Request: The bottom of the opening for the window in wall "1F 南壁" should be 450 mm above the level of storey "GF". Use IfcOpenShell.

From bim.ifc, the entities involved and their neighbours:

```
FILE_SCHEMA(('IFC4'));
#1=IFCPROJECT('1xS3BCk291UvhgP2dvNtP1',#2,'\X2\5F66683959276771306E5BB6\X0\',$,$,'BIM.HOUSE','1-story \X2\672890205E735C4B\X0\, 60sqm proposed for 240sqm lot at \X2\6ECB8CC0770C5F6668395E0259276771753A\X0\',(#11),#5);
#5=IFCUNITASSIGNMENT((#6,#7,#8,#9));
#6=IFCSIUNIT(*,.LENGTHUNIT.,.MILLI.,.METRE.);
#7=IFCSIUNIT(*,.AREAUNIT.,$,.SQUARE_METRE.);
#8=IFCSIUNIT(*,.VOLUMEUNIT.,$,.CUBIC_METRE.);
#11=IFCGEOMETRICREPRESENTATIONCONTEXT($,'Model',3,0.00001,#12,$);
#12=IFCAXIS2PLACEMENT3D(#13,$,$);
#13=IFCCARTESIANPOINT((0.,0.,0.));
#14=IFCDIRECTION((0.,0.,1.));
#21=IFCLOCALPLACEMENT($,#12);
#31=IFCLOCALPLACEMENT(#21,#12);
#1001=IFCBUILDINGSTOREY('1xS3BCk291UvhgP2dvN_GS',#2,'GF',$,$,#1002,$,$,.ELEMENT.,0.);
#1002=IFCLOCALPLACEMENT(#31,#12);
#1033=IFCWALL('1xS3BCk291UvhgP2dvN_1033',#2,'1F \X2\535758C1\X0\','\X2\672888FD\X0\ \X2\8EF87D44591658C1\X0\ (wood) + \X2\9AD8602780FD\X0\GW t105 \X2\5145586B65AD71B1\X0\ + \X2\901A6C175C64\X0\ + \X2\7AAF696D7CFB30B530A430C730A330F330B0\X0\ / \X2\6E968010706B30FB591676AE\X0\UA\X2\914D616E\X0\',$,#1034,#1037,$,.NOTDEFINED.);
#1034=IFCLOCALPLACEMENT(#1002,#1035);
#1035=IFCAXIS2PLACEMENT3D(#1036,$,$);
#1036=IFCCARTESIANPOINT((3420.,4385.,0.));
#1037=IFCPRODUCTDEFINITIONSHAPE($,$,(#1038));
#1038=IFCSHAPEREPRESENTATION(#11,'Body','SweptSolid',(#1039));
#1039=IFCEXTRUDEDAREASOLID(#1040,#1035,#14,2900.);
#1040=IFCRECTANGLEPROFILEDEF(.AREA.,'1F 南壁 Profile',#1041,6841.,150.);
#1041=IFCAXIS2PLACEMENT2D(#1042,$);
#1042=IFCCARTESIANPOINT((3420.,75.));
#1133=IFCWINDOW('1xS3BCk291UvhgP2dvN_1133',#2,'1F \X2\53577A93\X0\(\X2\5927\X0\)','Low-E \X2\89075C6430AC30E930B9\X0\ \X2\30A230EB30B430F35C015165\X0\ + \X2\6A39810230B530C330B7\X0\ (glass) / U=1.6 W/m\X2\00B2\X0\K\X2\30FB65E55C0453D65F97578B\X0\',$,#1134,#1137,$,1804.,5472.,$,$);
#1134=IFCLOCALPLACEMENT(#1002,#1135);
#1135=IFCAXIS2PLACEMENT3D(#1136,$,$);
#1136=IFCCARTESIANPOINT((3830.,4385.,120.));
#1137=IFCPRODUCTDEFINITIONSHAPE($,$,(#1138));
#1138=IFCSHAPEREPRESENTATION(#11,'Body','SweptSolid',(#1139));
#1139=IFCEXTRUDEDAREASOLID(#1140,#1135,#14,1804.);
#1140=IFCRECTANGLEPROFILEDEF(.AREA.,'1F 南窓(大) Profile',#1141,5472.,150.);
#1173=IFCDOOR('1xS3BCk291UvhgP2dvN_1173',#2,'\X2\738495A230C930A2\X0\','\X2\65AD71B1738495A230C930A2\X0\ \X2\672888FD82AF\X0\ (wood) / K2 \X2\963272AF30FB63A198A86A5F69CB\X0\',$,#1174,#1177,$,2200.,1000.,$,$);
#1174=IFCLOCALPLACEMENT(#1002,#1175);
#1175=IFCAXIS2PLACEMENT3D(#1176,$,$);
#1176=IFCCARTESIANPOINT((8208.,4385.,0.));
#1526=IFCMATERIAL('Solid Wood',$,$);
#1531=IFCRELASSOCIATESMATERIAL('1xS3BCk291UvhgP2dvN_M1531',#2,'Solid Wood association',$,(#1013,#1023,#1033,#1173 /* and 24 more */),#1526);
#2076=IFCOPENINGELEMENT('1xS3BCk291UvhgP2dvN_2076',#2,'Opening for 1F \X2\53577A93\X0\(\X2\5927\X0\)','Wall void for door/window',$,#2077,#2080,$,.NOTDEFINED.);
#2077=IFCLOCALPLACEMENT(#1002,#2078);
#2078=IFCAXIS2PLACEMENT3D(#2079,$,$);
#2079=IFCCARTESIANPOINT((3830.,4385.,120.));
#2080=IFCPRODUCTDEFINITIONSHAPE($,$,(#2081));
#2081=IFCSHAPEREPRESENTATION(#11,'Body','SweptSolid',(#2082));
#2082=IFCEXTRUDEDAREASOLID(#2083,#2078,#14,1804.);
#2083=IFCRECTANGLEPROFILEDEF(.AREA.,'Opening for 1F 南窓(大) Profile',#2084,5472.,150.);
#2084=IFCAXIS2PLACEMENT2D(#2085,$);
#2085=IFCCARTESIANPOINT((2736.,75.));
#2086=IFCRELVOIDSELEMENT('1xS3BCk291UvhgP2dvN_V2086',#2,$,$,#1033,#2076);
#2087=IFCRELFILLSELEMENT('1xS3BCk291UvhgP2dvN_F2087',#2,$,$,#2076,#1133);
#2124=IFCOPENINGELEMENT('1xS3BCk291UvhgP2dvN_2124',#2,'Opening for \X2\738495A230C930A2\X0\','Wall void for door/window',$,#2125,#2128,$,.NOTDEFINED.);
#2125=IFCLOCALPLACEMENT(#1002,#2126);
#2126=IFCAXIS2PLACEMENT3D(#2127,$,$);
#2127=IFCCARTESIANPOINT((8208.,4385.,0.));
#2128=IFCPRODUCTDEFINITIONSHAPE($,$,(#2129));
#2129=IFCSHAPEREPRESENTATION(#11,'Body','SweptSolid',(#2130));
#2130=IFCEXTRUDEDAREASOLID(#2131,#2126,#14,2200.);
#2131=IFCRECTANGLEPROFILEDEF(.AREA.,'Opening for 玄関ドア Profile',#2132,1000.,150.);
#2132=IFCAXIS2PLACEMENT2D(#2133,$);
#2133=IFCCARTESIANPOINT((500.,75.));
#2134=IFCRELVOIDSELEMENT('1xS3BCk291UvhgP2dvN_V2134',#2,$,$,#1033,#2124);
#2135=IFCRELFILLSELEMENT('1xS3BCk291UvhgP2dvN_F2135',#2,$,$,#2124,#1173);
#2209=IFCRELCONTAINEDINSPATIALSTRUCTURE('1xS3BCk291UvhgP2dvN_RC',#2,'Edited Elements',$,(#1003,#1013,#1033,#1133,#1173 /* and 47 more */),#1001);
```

```python
import numpy as np
import ifcopenshell
import ifcopenshell.api.geometry
import ifcopenshell.geom
import ifcopenshell.util.element
import ifcopenshell.util.placement
import ifcopenshell.util.shape
import ifcopenshell.util.unit

model = ifcopenshell.open("bim.ifc")
unit_scale = ifcopenshell.util.unit.calculate_unit_scale(model)

window = model.by_id(1133)
opening = window.FillsVoids[0].RelatingOpeningElement
storey = ifcopenshell.util.element.get_container(window, ifc_class="IfcBuildingStorey")
level = ifcopenshell.util.placement.get_local_placement(storey.ObjectPlacement)[2, 3]

# The opening's origin need not be at the sill, so measure its lowest point.
shape = ifcopenshell.geom.create_shape(ifcopenshell.geom.settings(), opening)
bottom = ifcopenshell.util.shape.get_shape_bottom_elevation(shape, shape.geometry) / unit_scale
dz = level + 0.45 / unit_scale - bottom

shift = np.array([0.0, 0.0, dz])
# The window is not placed relative to its opening, so move both.
for product in (opening, window):
    matrix = ifcopenshell.util.placement.get_local_placement(product.ObjectPlacement)
    matrix[:3, 3] += shift
    ifcopenshell.api.geometry.edit_object_placement(model, product=product, matrix=matrix, is_si=False)

print(f"moved by {dz * unit_scale:+.3f} m")

model.write("bim_v2.ifc")
```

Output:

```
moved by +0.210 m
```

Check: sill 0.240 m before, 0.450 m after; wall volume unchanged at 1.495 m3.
